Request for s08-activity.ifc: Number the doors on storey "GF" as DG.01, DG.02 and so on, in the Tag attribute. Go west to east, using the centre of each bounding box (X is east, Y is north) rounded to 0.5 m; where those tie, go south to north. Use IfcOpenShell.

First a look at what the model holds.

```python
import ifcopenshell
import ifcopenshell.util.element
import ifcopenshell.util.placement

model = ifcopenshell.open("s08-activity.ifc")
print(model.schema)
storey = next(s for s in model.by_type("IfcBuildingStorey") if s.Name == "GF")
doors = [e for e in ifcopenshell.util.element.get_decomposition(storey) if e.is_a("IfcDoor")]
for e in sorted(doors, key=lambda e: e.id()):
    origin = ifcopenshell.util.placement.get_local_placement(e.ObjectPlacement)[:3, 3]
    print(e.id(), e.Tag, e.Name, origin.round(2) + 0.0, sep=" | ")
```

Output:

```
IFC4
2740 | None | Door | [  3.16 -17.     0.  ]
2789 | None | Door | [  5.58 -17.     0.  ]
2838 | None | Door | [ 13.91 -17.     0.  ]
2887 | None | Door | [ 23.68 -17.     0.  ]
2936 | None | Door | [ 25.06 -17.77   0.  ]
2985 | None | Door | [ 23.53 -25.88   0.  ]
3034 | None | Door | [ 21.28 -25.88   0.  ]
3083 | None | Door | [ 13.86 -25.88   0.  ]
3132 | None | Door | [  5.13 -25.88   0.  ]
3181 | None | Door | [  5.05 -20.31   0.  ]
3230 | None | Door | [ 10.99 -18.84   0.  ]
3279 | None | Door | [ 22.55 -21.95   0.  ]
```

```python
import ifcopenshell
import ifcopenshell.geom
import ifcopenshell.util.element
import ifcopenshell.util.shape

model = ifcopenshell.open("s08-activity.ifc")
settings = ifcopenshell.geom.settings()
settings.set("use-world-coords", True)


def centre(element):
    shape = ifcopenshell.geom.create_shape(settings, element)
    return ifcopenshell.util.shape.get_bbox_centroid(shape.geometry)


storey = next(s for s in model.by_type("IfcBuildingStorey") if s.Name == "GF")
doors = [e for e in ifcopenshell.util.element.get_decomposition(storey) if e.is_a("IfcDoor")]

# Insertion points can sit at a corner or the storey origin, so sort by the geometry (in metres).
centres = {e: centre(e) for e in doors}
doors.sort(key=lambda e: (round(centres[e][0] / 0.5), centres[e][1]))

for i, e in enumerate(doors, start=1):
    number = f"DG.{i:02d}"
    e.Tag = number
    print(e.id(), number)

model.write("s08-activity_rev.ifc")
```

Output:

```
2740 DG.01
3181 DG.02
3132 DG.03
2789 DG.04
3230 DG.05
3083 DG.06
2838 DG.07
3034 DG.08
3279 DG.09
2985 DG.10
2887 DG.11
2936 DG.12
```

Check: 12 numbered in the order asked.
